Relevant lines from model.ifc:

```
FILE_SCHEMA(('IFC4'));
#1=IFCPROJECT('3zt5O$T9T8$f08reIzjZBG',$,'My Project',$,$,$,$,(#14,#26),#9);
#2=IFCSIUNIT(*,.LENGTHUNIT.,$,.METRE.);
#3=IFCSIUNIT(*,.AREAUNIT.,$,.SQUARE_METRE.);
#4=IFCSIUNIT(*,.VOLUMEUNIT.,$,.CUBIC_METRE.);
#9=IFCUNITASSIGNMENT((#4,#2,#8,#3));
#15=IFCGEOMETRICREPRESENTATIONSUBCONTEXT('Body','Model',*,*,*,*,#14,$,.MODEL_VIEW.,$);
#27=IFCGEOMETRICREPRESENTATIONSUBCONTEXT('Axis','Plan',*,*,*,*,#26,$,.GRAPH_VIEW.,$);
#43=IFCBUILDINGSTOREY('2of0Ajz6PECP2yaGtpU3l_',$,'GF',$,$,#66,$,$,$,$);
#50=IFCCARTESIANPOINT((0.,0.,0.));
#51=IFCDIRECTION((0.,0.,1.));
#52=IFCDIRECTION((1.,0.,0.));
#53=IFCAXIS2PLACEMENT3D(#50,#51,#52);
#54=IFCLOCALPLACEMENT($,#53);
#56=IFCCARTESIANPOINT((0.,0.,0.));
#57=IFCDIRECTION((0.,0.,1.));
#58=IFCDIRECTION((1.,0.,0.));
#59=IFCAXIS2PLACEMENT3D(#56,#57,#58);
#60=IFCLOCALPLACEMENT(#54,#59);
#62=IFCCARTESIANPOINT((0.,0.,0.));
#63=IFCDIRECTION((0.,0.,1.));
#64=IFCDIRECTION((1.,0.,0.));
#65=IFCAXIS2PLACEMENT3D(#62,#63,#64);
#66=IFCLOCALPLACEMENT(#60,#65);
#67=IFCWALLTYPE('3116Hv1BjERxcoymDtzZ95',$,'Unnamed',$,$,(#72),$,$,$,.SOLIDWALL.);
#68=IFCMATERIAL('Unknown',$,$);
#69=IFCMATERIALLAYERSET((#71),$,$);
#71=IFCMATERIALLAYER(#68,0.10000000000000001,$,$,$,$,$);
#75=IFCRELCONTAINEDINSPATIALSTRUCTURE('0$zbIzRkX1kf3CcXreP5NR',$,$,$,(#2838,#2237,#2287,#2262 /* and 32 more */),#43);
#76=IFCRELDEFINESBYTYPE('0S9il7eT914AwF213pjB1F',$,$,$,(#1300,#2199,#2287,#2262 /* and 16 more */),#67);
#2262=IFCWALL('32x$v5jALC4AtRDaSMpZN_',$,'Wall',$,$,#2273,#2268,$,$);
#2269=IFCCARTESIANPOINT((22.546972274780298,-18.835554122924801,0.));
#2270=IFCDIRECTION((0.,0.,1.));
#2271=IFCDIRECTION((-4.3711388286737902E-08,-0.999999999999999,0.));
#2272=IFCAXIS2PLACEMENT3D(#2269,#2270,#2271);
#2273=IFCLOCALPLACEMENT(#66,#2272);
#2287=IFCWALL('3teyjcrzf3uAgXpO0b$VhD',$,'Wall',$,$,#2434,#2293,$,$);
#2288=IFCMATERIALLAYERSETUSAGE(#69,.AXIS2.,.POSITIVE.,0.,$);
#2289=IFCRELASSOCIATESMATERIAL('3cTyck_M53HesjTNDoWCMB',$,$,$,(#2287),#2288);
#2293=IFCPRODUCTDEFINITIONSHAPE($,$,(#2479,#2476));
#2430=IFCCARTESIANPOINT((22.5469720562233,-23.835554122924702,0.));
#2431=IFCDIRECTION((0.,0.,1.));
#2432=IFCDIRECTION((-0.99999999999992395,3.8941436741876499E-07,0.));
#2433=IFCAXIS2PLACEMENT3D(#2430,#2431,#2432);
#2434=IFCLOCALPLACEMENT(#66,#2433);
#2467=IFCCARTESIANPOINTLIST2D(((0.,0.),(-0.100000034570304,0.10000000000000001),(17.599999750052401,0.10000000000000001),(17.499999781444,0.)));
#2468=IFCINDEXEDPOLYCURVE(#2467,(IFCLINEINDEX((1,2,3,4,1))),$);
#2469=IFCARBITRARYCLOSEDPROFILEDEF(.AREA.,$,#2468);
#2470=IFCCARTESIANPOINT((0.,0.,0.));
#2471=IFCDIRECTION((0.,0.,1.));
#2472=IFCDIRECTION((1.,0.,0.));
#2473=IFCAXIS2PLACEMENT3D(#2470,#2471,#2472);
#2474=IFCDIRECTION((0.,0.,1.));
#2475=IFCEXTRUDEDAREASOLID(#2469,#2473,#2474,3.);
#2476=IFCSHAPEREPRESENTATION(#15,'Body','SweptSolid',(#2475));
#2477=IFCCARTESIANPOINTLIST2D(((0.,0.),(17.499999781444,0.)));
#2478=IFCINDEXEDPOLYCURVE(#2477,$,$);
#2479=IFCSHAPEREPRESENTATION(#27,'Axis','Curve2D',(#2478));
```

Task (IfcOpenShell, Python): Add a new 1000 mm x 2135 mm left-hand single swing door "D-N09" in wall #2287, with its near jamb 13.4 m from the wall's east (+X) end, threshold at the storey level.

```python
import numpy as np
import ifcopenshell
import ifcopenshell.api.feature
import ifcopenshell.api.geometry
import ifcopenshell.api.root
import ifcopenshell.api.spatial
import ifcopenshell.geom
import ifcopenshell.util.element
import ifcopenshell.util.placement
import ifcopenshell.util.representation
import ifcopenshell.util.shape
import ifcopenshell.util.unit

model = ifcopenshell.open("model.ifc")
unit_scale = ifcopenshell.util.unit.calculate_unit_scale(model)
settings = ifcopenshell.geom.settings()


def volume(element):
    """Net volume in cubic metres, openings subtracted."""
    shape = ifcopenshell.geom.create_shape(settings, element)
    return ifcopenshell.util.shape.get_volume(shape.geometry)


wall = model.by_guid("3teyjcrzf3uAgXpO0b$VhD")
storey = ifcopenshell.util.element.get_container(wall, ifc_class="IfcBuildingStorey")
context = ifcopenshell.util.representation.get_context(model, "Model", "Body", "MODEL_VIEW")
before = volume(wall)

width, height, from_end, sill = 1, 2.135, 13.4, 0.0  # metres

# The wall runs along its own X axis, and the end named is its -X end.
wall_shape = ifcopenshell.geom.create_shape(settings, wall)
x, y, z = ifcopenshell.util.shape.get_vertices(wall_shape.geometry).T
start = x.min() + from_end
face, thickness = float(y.min()), float(y.max() - y.min())
wall_matrix = ifcopenshell.util.placement.get_local_placement(wall.ObjectPlacement)
level = ifcopenshell.util.placement.get_local_placement(storey.ObjectPlacement)[2, 3]


def in_wall(x, y):
    """Placement at x, y metres in the wall's axes, at sill height."""
    matrix = wall_matrix.copy()
    matrix[:, 3] = wall_matrix @ np.array([x / unit_scale, y / unit_scale, 0.0, 1.0])
    matrix[2, 3] = level + sill / unit_scale
    return matrix


# Opening: a box that overshoots both wall faces by 50 mm.
opening = ifcopenshell.api.root.create_entity(model, ifc_class="IfcOpeningElement", predefined_type="OPENING")
box = ifcopenshell.api.geometry.add_wall_representation(
    model, context=context, length=width, height=height, thickness=thickness + 0.1
)
ifcopenshell.api.geometry.assign_representation(model, product=opening, representation=box)
ifcopenshell.api.geometry.edit_object_placement(model, product=opening, matrix=in_wall(start, face - 0.05), is_si=False)
ifcopenshell.api.feature.add_feature(model, feature=opening, element=wall)

door = ifcopenshell.api.root.create_entity(model, ifc_class="IfcDoor", name="D-N09", predefined_type="DOOR")
door.OverallWidth, door.OverallHeight = width / unit_scale, height / unit_scale
door.OperationType = "SINGLE_SWING_LEFT"
body = ifcopenshell.api.geometry.add_door_representation(
    model,
    context=context,
    overall_width=door.OverallWidth,
    overall_height=door.OverallHeight,
    operation_type="SINGLE_SWING_LEFT",
    lining_properties={"LiningDepth": thickness / unit_scale, "ThresholdDepth": thickness / unit_scale},
)
ifcopenshell.api.geometry.assign_representation(model, product=door, representation=body)
ifcopenshell.api.spatial.assign_container(model, products=[door], relating_structure=storey)
ifcopenshell.api.feature.add_filling(model, opening=opening, element=door)

# The lining spans the wall, so the door starts at the wall face.
ifcopenshell.api.geometry.edit_object_placement(model, product=door, matrix=in_wall(start, face), is_si=False)

after = volume(wall)

print(f"wall volume {before:.3f} -> {after:.3f} m3")

model.write("model_v2.ifc")
```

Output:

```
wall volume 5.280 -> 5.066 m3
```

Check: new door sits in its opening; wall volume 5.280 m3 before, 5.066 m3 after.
